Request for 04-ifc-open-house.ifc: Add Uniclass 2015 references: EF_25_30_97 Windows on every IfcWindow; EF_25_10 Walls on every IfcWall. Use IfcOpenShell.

First a look at what the model holds.

```python
import ifcopenshell

model = ifcopenshell.open("04-ifc-open-house.ifc")
print(model.schema)
print("classifications:", [c.Name for c in model.by_type("IfcClassification")])
for ifc_class in ("IfcDoor", "IfcRoof", "IfcStair", "IfcWall", "IfcWindow"):
    print(ifc_class, len(model.by_type(ifc_class)))
```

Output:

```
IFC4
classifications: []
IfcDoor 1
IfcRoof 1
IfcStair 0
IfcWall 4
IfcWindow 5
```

```python
import ifcopenshell
import ifcopenshell.api.classification

model = ifcopenshell.open("04-ifc-open-house.ifc")

system = ifcopenshell.api.classification.add_classification(model, classification="Uniclass 2015")

codes = {
    "IfcWindow": ("EF_25_30_97", "Windows"),
    "IfcWall": ("EF_25_10", "Walls"),
}
for ifc_class, (code, name) in codes.items():
    products = model.by_type(ifc_class)
    ifcopenshell.api.classification.add_reference(
        model, products=products, classification=system, identification=code, name=name
    )
    print(code, len(products))

model.write("04-ifc-open-house_v2.ifc")
```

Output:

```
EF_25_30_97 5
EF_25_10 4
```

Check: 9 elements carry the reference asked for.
